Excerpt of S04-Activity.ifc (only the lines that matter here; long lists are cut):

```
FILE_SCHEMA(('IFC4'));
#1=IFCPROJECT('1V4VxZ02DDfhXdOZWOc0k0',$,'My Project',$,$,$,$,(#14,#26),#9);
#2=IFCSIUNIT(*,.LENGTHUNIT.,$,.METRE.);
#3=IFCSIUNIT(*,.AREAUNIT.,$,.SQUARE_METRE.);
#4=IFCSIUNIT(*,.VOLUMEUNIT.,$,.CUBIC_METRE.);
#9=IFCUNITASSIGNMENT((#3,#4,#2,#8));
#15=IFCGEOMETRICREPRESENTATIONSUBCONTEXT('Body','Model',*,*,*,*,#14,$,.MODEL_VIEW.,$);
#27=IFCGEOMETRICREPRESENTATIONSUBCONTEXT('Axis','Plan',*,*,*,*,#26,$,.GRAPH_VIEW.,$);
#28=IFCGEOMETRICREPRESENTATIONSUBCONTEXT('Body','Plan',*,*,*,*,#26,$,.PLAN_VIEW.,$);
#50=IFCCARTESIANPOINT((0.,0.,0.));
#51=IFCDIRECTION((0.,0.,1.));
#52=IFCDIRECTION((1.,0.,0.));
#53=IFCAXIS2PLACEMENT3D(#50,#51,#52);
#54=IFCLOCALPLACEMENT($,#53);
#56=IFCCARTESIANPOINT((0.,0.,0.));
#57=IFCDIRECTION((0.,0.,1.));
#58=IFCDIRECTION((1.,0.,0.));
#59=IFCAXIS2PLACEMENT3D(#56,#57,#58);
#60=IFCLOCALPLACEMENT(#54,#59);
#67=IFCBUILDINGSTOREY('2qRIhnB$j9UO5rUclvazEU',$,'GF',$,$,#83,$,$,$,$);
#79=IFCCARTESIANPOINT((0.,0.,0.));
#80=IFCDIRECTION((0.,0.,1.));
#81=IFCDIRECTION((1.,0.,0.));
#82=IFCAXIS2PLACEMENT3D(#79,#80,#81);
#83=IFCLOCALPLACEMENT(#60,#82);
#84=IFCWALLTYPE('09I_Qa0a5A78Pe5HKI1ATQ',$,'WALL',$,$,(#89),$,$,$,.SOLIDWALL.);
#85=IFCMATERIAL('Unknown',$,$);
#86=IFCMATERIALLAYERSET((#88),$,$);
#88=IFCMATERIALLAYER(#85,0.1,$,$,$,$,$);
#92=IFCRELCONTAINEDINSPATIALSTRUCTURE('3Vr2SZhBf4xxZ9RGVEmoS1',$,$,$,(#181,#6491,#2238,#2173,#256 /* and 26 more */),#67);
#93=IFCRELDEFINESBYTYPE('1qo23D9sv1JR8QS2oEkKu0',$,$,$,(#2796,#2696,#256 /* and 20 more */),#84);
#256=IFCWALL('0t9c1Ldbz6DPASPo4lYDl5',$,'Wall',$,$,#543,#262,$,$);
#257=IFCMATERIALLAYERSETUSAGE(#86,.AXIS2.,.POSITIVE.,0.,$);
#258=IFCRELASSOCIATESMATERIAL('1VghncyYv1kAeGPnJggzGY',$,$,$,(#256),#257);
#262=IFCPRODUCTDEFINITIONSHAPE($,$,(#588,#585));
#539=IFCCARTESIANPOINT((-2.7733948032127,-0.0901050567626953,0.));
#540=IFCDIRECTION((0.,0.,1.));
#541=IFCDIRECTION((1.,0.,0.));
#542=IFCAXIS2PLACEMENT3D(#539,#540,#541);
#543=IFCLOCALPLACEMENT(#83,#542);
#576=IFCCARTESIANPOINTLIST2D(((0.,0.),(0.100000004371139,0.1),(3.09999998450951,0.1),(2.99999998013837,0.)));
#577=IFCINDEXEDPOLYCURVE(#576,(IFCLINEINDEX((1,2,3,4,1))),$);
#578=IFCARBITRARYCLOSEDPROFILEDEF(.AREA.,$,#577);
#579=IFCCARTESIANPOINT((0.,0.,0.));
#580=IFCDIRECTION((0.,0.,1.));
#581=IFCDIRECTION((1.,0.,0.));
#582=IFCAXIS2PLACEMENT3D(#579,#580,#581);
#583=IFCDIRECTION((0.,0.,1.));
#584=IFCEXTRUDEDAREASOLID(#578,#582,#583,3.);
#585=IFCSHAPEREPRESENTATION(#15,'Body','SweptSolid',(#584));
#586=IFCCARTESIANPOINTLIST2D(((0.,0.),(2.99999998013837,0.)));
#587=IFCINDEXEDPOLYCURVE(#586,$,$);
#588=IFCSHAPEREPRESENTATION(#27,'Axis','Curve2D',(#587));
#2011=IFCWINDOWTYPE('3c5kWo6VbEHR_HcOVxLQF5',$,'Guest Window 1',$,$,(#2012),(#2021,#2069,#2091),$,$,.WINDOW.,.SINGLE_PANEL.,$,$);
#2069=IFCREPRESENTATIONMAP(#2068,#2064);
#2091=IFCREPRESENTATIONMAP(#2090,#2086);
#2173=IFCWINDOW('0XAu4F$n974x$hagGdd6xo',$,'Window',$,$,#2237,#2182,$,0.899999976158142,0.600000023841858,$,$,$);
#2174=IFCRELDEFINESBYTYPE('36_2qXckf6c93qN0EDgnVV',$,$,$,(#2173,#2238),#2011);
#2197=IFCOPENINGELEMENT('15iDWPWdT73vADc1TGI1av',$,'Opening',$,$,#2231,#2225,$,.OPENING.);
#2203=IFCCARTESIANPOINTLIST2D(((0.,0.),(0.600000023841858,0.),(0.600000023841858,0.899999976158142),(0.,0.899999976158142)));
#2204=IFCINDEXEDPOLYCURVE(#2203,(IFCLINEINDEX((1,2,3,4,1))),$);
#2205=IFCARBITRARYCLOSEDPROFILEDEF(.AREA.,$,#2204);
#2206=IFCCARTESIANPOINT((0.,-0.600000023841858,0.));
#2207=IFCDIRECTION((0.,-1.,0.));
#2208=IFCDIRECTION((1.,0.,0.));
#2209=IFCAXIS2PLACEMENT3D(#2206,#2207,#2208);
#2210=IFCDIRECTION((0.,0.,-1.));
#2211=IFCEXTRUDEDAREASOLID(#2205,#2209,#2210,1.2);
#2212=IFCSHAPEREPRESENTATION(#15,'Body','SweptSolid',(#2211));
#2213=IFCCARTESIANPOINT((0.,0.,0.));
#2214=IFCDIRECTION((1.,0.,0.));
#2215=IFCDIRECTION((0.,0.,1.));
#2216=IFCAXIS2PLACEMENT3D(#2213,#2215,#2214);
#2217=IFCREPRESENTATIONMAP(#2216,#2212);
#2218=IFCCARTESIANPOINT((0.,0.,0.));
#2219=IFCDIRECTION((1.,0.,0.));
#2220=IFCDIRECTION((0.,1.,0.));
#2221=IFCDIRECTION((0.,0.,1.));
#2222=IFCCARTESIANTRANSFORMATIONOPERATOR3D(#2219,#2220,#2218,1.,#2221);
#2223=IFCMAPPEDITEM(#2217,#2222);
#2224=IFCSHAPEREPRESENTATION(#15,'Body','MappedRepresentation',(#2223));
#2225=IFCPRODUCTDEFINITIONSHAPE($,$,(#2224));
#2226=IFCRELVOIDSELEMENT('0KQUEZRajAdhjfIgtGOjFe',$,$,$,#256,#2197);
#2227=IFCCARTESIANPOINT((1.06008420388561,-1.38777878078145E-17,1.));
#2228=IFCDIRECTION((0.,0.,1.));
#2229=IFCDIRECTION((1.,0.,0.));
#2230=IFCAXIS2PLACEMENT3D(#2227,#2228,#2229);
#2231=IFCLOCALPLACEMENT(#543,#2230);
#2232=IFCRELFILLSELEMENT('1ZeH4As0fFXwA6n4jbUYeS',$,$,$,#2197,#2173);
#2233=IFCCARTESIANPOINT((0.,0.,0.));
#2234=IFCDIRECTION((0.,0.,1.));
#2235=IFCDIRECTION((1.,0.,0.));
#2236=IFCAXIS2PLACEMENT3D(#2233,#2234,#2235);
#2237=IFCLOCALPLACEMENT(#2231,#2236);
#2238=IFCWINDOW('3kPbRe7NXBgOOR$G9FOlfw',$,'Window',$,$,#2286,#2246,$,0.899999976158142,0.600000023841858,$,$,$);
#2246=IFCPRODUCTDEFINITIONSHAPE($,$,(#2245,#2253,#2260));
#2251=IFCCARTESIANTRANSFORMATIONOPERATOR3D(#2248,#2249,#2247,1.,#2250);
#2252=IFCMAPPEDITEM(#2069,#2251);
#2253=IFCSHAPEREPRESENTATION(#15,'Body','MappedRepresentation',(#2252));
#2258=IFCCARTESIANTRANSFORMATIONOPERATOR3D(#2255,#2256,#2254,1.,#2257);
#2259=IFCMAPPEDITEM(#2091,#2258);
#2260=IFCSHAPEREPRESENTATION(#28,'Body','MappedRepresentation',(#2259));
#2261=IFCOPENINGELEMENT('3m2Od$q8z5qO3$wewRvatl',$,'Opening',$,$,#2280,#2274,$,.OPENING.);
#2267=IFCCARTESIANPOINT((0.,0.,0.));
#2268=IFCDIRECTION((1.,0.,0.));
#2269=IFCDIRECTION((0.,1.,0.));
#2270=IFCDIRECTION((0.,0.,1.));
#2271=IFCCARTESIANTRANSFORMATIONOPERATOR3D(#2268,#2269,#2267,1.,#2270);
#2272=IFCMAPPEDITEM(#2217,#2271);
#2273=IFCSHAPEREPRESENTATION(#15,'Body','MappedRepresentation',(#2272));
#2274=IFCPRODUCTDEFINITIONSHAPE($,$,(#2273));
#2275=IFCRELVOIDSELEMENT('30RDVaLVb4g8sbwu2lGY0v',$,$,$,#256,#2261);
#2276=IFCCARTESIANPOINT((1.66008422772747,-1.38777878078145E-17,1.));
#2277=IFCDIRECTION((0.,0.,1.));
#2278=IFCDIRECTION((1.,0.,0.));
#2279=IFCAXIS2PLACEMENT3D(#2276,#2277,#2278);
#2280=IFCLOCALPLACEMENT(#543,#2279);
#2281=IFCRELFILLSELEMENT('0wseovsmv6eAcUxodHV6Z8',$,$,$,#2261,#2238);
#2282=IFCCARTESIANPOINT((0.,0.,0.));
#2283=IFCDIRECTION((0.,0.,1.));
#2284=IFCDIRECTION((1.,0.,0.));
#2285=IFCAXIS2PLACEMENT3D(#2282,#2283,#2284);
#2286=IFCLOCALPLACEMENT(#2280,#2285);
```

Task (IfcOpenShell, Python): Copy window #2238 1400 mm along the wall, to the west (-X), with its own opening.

```python
import ifcopenshell
import ifcopenshell.api.feature
import ifcopenshell.api.geometry
import ifcopenshell.api.root
import ifcopenshell.geom
import ifcopenshell.util.element
import ifcopenshell.util.placement
import ifcopenshell.util.shape
import ifcopenshell.util.unit

model = ifcopenshell.open("S04-Activity.ifc")
unit_scale = ifcopenshell.util.unit.calculate_unit_scale(model)
settings = ifcopenshell.geom.settings()


def volume(element):
    """Net volume in cubic metres, openings subtracted."""
    shape = ifcopenshell.geom.create_shape(settings, element)
    return ifcopenshell.util.shape.get_volume(shape.geometry)


window = model.by_guid("3kPbRe7NXBgOOR$G9FOlfw")
opening = window.FillsVoids[0].RelatingOpeningElement
wall = opening.VoidsElements[0].RelatingBuildingElement
before = volume(wall)
shift = ifcopenshell.util.placement.get_local_placement(wall.ObjectPlacement)[:3, 0] * -1.4 / unit_scale

# copy_class copies the void relationship, type, container and properties, but no geometry.
new_opening = ifcopenshell.api.root.copy_class(model, product=opening)
new_opening.Representation = ifcopenshell.util.element.copy_deep(
    model, opening.Representation, exclude=["IfcGeometricRepresentationContext", "IfcRepresentationMap"]
)
new_window = ifcopenshell.api.root.copy_class(model, product=window)
new_window.Representation = ifcopenshell.util.element.copy_deep(
    model, window.Representation, exclude=["IfcGeometricRepresentationContext", "IfcRepresentationMap"]
)
ifcopenshell.api.feature.add_filling(model, opening=new_opening, element=new_window)

for old, new in ((opening, new_opening), (window, new_window)):
    matrix = ifcopenshell.util.placement.get_local_placement(old.ObjectPlacement)
    matrix[:3, 3] += shift
    ifcopenshell.api.geometry.edit_object_placement(model, product=new, matrix=matrix, is_si=False)

after = volume(wall)

print(f"wall volume {before:.3f} -> {after:.3f} m3")

model.write("S04-Activity_edited.ifc")
```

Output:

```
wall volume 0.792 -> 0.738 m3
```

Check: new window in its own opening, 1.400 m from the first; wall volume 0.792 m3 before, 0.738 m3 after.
